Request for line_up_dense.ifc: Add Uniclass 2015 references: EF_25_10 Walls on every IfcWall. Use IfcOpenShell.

First a look at what the model holds.

```python
import ifcopenshell

model = ifcopenshell.open("line_up_dense.ifc")
print(model.schema)
print("classifications:", [c.Name for c in model.by_type("IfcClassification")])
for ifc_class in ("IfcDoor", "IfcRoof", "IfcStair", "IfcWall", "IfcWindow"):
    print(ifc_class, len(model.by_type(ifc_class)))
```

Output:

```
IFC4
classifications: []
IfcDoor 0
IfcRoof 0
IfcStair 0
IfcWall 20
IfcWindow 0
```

```python
import ifcopenshell
import ifcopenshell.api.classification

model = ifcopenshell.open("line_up_dense.ifc")

system = ifcopenshell.api.classification.add_classification(model, classification="Uniclass 2015")

codes = {
    "IfcWall": ("EF_25_10", "Walls"),
}
for ifc_class, (code, name) in codes.items():
    products = model.by_type(ifc_class)
    ifcopenshell.api.classification.add_reference(
        model, products=products, classification=system, identification=code, name=name
    )
    print(code, len(products))

model.write("line_up_dense_rev.ifc")
```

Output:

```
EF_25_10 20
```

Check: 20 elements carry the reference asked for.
